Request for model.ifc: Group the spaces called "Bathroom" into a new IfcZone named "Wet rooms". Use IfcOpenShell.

First a look at what the model holds.

```python
import ifcopenshell

model = ifcopenshell.open("model.ifc")
print(model.schema)
seen = {}
for space in model.by_type("IfcSpace"):
    seen[space.Name] = seen.get(space.Name, 0) + 1
for name, count in sorted(seen.items(), key=str):
    print(count, "x", name)
print("zones:", [z.Name for z in model.by_type("IfcZone")][:20])
```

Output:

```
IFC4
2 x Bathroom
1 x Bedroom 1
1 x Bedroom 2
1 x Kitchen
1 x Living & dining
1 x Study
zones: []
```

```python
import ifcopenshell
import ifcopenshell.api.group
import ifcopenshell.api.root

model = ifcopenshell.open("model.ifc")

names = {"Bathroom"}
spaces = [s for s in model.by_type("IfcSpace") if s.Name in names]

zone = ifcopenshell.api.root.create_entity(model, ifc_class="IfcZone", name="Wet rooms")
ifcopenshell.api.group.assign_group(model, products=spaces, group=zone)
print(len(spaces), "spaces in", zone.Name)

model.write("model_updated.ifc")
```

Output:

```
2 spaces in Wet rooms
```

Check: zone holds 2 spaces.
